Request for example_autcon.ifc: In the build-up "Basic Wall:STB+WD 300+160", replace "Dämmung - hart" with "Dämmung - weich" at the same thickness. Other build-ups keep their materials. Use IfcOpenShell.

First a look at what the model holds.

```python
import ifcopenshell
import ifcopenshell.util.element

model = ifcopenshell.open("example_autcon.ifc")
print(model.schema)
for layer_set in model.by_type("IfcMaterialLayerSet"):
    if layer_set.LayerSetName == "Basic Wall:STB+WD 300+160":
        for layer in layer_set.MaterialLayers:
            print(layer.id(), layer.Material and layer.Material.Name, layer.LayerThickness, sep=" | ")
        print(len(ifcopenshell.util.element.get_elements_by_material(model, layer_set)), "elements and types use it")
print(sorted(m.Name for m in model.by_type("IfcMaterial") if m.Name)[:60])
```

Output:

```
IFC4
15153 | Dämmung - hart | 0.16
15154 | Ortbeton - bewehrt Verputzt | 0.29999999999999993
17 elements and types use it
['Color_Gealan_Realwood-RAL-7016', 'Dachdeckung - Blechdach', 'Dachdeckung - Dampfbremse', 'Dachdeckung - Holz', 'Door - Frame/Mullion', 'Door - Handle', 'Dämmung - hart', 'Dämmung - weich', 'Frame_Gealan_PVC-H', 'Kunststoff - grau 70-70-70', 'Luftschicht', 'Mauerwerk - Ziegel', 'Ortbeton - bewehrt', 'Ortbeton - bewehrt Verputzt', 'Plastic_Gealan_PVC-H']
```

```python
import ifcopenshell
import ifcopenshell.api.material

model = ifcopenshell.open("example_autcon.ifc")

layer_set = next(s for s in model.by_type("IfcMaterialLayerSet") if s.LayerSetName == "Basic Wall:STB+WD 300+160")
layer = next(l for l in layer_set.MaterialLayers if l.Material and l.Material.Name == "Dämmung - hart")
material = next(m for m in model.by_type("IfcMaterial") if m.Name == "Dämmung - weich")

# Point this one layer at the other material; renaming the old one would change it everywhere.
ifcopenshell.api.material.edit_layer(model, layer=layer, attributes={"Name": material.Name}, material=material)

print([l.Material.Name if l.Material else None for l in layer_set.MaterialLayers])

model.write("example_autcon-out.ifc")
```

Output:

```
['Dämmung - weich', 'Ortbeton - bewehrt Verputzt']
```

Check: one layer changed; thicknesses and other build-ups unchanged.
